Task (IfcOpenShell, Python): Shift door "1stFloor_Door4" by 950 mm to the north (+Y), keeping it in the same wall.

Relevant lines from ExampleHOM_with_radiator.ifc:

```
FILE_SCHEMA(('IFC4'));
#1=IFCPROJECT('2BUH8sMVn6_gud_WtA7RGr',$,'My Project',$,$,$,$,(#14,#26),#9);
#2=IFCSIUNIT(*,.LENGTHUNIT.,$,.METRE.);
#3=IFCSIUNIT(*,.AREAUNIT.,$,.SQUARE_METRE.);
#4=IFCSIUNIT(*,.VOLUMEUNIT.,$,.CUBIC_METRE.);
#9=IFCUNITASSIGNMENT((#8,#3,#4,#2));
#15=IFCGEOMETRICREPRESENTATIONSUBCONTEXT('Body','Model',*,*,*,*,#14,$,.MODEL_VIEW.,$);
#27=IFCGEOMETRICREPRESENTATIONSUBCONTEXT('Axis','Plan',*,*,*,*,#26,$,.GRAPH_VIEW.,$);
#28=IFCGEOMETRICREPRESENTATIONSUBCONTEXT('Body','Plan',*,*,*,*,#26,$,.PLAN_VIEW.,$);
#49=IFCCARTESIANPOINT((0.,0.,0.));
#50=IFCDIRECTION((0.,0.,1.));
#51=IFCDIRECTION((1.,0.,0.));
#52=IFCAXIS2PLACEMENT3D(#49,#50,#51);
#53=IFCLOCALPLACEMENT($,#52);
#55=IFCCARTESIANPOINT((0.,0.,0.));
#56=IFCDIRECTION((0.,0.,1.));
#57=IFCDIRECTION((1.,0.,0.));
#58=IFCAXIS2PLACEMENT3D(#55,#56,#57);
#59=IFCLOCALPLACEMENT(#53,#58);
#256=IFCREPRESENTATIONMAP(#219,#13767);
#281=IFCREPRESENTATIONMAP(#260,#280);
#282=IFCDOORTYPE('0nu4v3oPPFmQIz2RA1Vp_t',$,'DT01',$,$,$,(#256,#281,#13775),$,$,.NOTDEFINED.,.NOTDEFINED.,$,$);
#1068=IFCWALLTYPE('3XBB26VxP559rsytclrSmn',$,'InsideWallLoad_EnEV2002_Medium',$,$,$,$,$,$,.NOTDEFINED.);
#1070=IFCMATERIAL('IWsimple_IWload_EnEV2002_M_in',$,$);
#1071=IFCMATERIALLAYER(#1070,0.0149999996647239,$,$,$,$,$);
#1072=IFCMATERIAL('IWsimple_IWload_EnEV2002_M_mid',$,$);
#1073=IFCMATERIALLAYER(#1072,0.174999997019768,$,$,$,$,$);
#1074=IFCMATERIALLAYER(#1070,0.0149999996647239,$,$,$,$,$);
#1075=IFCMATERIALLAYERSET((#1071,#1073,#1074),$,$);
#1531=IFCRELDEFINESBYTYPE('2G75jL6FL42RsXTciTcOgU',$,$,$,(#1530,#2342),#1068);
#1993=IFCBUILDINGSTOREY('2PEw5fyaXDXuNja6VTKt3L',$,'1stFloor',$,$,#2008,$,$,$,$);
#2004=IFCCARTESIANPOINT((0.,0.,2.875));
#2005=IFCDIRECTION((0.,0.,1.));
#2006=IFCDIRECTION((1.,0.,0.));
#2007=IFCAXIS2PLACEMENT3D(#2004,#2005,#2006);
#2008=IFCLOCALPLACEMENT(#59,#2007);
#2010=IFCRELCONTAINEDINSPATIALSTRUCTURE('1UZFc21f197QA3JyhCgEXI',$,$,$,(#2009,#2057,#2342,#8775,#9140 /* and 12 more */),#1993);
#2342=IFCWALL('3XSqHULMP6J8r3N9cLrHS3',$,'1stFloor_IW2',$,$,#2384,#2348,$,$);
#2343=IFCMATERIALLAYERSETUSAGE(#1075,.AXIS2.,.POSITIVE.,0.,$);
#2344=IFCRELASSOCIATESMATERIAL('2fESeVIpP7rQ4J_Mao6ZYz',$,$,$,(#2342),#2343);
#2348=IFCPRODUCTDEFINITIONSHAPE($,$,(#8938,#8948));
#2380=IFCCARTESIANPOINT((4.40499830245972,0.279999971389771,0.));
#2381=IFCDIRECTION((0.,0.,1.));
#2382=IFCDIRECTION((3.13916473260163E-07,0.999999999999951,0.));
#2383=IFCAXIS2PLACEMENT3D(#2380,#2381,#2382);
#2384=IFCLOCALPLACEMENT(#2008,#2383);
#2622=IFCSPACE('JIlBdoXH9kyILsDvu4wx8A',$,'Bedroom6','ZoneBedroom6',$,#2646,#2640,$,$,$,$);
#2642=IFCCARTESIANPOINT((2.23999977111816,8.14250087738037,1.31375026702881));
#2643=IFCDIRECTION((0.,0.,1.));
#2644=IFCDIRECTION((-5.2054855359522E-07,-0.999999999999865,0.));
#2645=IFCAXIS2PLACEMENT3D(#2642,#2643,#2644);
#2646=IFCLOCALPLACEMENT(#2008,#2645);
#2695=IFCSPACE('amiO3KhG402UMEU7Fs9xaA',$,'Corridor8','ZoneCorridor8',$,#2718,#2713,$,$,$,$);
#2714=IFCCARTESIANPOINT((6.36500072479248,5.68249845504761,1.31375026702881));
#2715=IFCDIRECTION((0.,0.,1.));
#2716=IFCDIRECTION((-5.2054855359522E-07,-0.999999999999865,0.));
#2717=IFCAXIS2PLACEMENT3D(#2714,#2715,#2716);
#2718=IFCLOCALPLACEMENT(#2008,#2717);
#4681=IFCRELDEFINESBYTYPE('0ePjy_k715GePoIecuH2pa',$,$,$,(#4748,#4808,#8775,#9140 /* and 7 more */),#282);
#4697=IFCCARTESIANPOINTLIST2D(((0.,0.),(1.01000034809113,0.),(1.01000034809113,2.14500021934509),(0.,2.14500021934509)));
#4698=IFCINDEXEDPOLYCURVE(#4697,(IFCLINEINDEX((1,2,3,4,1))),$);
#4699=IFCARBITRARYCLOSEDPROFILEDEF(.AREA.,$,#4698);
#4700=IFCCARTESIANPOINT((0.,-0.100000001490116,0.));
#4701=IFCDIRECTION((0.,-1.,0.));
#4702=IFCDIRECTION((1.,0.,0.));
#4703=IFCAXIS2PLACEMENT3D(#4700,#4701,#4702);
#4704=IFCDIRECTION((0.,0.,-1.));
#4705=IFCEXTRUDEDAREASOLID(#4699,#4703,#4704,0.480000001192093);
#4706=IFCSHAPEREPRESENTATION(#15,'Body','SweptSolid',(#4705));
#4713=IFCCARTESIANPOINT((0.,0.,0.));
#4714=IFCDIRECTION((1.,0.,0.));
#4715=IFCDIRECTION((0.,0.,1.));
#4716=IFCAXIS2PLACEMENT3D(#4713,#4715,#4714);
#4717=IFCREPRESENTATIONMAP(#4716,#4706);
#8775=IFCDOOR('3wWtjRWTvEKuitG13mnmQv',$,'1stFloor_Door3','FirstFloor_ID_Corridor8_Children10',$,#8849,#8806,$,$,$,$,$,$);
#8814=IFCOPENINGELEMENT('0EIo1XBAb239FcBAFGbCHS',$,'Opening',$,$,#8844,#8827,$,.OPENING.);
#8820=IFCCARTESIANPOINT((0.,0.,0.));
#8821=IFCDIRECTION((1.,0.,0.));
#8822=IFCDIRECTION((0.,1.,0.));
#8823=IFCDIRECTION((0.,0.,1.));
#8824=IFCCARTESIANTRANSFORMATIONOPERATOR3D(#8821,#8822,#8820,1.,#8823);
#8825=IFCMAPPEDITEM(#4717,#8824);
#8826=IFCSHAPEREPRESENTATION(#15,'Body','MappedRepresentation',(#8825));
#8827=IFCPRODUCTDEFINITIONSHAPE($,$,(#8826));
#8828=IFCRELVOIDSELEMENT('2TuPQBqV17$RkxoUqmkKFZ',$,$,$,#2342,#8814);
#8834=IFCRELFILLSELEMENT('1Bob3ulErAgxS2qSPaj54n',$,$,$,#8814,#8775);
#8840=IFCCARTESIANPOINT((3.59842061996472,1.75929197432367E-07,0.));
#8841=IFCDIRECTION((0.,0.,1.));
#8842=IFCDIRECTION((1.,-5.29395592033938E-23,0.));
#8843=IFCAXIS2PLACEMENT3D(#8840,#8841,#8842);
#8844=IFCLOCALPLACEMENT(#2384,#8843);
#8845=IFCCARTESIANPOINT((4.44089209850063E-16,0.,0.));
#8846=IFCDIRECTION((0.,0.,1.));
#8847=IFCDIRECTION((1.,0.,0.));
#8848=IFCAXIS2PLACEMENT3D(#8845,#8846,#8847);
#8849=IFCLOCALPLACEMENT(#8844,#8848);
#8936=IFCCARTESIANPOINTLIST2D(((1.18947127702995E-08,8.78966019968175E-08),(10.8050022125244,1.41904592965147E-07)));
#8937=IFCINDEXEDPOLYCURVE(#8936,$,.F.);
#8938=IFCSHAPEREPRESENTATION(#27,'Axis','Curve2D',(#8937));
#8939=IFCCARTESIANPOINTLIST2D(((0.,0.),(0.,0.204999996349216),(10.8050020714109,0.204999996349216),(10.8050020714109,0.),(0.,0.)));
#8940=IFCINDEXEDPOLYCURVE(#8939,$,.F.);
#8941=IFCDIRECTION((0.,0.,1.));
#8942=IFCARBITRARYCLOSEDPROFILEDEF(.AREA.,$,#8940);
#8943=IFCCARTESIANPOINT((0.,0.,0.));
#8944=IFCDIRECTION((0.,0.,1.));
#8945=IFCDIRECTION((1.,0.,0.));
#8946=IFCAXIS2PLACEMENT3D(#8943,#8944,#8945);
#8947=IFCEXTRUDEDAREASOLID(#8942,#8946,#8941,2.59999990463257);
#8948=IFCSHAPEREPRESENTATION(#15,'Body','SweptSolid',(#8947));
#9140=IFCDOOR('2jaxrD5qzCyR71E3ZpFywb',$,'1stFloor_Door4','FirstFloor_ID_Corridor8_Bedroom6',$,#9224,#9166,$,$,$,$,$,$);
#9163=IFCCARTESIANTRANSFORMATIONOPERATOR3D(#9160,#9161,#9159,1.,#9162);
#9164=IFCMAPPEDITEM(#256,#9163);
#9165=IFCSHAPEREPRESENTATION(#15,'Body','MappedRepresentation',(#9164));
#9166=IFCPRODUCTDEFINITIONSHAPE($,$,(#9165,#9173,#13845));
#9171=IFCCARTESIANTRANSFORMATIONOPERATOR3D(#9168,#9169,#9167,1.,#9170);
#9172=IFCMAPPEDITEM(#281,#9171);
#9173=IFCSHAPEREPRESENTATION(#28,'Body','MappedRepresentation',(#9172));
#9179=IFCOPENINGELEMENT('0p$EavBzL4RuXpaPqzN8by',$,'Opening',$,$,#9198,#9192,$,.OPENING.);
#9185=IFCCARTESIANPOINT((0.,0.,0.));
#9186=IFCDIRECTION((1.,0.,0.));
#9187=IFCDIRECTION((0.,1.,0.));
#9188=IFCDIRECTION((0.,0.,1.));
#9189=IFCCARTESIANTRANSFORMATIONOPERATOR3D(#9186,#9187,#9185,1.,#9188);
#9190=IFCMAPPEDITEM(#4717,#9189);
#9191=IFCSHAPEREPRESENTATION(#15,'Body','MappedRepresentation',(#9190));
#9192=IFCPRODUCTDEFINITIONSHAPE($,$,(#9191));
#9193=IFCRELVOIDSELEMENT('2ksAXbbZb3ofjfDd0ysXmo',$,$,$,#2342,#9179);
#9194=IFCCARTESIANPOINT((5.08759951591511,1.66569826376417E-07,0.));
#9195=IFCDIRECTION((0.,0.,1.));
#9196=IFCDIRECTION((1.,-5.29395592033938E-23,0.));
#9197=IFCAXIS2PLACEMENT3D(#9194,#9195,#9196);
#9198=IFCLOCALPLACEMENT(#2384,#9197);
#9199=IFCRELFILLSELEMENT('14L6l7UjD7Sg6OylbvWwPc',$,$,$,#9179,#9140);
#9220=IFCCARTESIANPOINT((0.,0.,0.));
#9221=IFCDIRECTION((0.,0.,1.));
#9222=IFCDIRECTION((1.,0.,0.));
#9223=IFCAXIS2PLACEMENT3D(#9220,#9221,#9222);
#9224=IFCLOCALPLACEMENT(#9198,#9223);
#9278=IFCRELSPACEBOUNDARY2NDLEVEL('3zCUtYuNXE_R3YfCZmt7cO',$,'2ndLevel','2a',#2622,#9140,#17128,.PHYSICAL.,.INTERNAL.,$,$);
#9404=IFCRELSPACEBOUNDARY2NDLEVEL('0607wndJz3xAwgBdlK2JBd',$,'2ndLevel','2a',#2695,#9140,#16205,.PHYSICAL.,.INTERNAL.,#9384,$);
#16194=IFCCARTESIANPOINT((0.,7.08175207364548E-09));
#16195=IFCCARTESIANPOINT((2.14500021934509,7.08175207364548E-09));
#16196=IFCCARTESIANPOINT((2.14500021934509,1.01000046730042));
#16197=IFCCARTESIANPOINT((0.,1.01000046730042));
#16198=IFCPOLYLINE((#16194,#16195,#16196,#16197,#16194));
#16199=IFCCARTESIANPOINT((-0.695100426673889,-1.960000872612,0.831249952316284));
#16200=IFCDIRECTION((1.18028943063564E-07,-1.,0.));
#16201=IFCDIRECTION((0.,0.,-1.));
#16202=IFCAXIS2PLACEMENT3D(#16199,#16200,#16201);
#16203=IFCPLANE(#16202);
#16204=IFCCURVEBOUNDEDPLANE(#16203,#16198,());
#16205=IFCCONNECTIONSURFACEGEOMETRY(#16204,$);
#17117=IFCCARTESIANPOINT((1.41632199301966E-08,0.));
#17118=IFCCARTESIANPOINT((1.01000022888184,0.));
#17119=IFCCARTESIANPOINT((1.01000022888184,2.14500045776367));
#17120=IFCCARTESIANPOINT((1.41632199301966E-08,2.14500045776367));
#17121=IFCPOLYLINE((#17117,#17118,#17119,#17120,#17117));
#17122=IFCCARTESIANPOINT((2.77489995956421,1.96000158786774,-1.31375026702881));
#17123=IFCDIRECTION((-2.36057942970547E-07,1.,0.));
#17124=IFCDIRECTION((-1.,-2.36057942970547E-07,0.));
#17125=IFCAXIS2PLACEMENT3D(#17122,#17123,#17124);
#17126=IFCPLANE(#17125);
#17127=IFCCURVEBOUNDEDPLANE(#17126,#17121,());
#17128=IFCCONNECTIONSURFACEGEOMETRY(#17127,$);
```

```python
import numpy as np
import ifcopenshell
import ifcopenshell.api.geometry
import ifcopenshell.util.placement
import ifcopenshell.util.unit

model = ifcopenshell.open("ExampleHOM_with_radiator.ifc")
unit_scale = ifcopenshell.util.unit.calculate_unit_scale(model)

door = model.by_guid("2jaxrD5qzCyR71E3ZpFywb")
opening = door.FillsVoids[0].RelatingOpeningElement
wall = opening.VoidsElements[0].RelatingBuildingElement

wall_matrix = ifcopenshell.util.placement.get_local_placement(wall.ObjectPlacement)
shift = wall_matrix[:3, 0] * 0.95 / unit_scale
before = ifcopenshell.util.placement.get_local_placement(door.ObjectPlacement)[:3, 3].copy()

# The door is placed relative to its opening, so it follows when the opening moves.
matrix = ifcopenshell.util.placement.get_local_placement(opening.ObjectPlacement)
matrix[:3, 3] += shift
ifcopenshell.api.geometry.edit_object_placement(
    model, product=opening, matrix=matrix, is_si=False, should_transform_children=True
)

# Space boundary surfaces are stored in each space's coordinates; move them too.
for rel in door.ProvidesBoundaries:
    if not rel.ConnectionGeometry:
        continue
    surface = rel.ConnectionGeometry.SurfaceOnRelatingElement.BasisSurface
    space_matrix = ifcopenshell.util.placement.get_local_placement(rel.RelatingSpace.ObjectPlacement)
    point = np.array(surface.Position.Location.Coordinates) + space_matrix[:3, :3].T @ shift
    surface.Position = model.createIfcAxis2Placement3D(
        model.createIfcCartesianPoint(point.tolist()), surface.Position.Axis, surface.Position.RefDirection
    )

after = ifcopenshell.util.placement.get_local_placement(door.ObjectPlacement)[:3, 3]
print("door moved by", (after - before).round(3) + 0.0)

model.write("ExampleHOM_with_radiator_v2.ifc")
```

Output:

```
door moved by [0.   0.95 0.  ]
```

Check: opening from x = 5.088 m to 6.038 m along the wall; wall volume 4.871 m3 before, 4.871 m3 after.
